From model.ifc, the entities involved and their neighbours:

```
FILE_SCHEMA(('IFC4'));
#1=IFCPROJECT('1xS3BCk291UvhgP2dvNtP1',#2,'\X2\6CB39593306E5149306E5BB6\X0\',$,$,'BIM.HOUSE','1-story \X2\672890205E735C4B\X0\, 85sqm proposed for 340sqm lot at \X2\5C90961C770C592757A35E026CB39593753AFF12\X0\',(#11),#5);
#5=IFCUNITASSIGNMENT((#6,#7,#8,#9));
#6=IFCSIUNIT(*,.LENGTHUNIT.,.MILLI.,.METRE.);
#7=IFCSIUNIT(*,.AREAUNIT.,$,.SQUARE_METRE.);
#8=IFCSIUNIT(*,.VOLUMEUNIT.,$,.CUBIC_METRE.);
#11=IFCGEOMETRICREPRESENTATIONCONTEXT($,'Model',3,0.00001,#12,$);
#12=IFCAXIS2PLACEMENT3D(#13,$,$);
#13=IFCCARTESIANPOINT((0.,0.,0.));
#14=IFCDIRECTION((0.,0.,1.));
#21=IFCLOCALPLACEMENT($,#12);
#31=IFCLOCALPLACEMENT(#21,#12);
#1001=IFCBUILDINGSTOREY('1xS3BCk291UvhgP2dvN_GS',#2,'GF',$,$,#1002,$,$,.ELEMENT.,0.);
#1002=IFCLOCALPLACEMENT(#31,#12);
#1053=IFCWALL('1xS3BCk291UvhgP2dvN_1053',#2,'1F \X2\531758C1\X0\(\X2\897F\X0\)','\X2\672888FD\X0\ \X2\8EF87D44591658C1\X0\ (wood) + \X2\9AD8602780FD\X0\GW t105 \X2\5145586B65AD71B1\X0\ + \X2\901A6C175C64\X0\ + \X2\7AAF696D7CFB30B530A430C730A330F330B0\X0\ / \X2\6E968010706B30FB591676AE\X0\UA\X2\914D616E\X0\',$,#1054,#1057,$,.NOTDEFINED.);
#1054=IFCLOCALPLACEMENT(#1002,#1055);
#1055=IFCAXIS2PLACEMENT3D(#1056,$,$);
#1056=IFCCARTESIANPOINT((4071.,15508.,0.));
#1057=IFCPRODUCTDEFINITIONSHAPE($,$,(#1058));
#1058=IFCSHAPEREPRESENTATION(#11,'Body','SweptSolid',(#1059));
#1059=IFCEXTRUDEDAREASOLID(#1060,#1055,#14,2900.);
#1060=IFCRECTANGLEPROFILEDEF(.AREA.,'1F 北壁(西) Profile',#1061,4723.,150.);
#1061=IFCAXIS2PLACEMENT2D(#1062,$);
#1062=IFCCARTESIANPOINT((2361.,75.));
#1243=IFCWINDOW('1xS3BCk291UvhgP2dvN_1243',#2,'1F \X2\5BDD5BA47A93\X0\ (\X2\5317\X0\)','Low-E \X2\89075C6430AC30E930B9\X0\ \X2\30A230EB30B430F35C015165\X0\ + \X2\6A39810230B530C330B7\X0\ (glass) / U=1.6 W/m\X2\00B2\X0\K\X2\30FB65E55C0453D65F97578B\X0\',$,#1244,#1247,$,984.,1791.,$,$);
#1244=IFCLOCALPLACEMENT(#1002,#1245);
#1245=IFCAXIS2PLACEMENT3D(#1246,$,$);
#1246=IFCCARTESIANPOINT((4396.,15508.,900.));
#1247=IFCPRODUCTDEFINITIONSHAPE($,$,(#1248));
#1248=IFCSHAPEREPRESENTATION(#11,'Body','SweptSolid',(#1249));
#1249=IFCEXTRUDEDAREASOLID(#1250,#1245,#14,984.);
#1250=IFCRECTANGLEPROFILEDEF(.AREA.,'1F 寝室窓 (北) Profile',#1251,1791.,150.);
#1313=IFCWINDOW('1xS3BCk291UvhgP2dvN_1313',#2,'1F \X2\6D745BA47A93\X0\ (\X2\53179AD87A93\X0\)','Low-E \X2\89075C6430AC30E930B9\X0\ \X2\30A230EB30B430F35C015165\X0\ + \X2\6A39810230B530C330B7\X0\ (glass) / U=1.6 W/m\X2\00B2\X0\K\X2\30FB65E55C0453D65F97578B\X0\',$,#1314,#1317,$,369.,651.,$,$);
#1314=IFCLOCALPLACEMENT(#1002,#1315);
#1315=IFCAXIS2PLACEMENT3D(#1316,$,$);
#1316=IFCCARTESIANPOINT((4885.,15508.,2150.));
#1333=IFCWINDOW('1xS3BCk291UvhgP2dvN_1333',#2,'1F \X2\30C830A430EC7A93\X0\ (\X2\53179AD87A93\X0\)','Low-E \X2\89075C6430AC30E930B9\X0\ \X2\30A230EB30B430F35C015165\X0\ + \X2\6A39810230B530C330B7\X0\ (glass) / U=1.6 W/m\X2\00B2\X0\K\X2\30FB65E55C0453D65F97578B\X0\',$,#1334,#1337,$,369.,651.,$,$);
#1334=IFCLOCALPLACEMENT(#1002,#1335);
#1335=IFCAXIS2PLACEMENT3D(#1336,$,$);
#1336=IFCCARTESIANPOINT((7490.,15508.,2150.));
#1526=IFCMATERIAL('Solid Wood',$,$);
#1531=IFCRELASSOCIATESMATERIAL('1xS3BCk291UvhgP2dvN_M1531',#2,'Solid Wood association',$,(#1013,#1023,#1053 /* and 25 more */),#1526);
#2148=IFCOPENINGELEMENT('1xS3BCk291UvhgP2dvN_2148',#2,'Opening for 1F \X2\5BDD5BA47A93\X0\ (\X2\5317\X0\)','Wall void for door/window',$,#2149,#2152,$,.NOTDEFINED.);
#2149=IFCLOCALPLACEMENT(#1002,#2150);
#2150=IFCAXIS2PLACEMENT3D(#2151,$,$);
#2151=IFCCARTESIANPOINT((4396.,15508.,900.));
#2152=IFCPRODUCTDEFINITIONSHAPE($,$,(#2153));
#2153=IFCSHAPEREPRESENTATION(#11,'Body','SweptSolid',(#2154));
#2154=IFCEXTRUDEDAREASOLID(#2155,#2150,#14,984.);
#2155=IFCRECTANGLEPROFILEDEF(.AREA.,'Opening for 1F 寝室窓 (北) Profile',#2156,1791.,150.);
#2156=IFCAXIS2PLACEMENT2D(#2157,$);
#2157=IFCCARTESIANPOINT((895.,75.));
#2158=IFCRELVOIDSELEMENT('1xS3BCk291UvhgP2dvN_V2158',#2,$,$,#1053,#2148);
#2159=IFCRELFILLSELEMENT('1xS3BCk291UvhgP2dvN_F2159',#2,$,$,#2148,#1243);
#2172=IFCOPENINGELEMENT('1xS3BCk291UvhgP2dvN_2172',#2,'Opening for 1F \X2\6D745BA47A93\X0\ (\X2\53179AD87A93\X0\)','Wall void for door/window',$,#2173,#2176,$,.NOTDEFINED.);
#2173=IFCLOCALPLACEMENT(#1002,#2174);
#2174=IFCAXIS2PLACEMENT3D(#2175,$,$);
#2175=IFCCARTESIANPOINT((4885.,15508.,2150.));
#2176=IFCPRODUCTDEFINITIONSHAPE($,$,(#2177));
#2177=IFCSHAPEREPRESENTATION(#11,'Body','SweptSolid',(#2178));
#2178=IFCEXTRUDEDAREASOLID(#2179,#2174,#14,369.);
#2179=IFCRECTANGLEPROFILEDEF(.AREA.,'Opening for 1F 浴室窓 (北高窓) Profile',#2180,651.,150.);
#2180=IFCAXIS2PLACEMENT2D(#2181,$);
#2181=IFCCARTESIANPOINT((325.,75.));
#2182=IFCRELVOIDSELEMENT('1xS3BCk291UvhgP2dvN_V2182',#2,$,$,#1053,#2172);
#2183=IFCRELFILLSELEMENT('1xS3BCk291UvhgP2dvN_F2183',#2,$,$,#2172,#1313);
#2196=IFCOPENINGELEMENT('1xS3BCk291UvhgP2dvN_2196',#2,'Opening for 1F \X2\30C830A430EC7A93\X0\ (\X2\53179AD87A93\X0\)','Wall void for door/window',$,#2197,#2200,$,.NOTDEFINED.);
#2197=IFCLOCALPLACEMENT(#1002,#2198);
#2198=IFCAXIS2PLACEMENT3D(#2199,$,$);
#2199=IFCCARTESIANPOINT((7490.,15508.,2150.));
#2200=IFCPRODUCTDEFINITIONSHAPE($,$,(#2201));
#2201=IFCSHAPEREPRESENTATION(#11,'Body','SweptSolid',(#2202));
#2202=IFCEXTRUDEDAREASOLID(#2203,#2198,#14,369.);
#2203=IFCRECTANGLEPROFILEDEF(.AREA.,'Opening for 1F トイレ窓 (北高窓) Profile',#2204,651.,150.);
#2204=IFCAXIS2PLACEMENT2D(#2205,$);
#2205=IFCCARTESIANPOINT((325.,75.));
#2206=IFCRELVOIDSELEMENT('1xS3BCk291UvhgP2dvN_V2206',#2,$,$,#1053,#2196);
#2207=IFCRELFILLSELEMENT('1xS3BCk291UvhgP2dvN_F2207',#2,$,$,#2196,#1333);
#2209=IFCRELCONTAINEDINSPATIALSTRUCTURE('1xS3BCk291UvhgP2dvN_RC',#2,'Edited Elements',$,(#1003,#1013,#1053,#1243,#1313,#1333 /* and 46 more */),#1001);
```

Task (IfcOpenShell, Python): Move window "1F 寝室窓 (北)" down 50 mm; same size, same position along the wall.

```python
import numpy as np
import ifcopenshell
import ifcopenshell.api.geometry
import ifcopenshell.util.placement
import ifcopenshell.util.unit

model = ifcopenshell.open("model.ifc")
unit_scale = ifcopenshell.util.unit.calculate_unit_scale(model)

window = model.by_guid("1xS3BCk291UvhgP2dvN_1243")
opening = window.FillsVoids[0].RelatingOpeningElement
dz = -50.0

shift = np.array([0.0, 0.0, dz])
# The window is not placed relative to its opening, so move both.
for product in (opening, window):
    matrix = ifcopenshell.util.placement.get_local_placement(product.ObjectPlacement)
    matrix[:3, 3] += shift
    ifcopenshell.api.geometry.edit_object_placement(model, product=product, matrix=matrix, is_si=False)

print(f"moved by {dz * unit_scale:+.3f} m")

model.write("model-out.ifc")
```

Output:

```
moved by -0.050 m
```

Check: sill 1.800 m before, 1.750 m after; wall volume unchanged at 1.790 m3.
